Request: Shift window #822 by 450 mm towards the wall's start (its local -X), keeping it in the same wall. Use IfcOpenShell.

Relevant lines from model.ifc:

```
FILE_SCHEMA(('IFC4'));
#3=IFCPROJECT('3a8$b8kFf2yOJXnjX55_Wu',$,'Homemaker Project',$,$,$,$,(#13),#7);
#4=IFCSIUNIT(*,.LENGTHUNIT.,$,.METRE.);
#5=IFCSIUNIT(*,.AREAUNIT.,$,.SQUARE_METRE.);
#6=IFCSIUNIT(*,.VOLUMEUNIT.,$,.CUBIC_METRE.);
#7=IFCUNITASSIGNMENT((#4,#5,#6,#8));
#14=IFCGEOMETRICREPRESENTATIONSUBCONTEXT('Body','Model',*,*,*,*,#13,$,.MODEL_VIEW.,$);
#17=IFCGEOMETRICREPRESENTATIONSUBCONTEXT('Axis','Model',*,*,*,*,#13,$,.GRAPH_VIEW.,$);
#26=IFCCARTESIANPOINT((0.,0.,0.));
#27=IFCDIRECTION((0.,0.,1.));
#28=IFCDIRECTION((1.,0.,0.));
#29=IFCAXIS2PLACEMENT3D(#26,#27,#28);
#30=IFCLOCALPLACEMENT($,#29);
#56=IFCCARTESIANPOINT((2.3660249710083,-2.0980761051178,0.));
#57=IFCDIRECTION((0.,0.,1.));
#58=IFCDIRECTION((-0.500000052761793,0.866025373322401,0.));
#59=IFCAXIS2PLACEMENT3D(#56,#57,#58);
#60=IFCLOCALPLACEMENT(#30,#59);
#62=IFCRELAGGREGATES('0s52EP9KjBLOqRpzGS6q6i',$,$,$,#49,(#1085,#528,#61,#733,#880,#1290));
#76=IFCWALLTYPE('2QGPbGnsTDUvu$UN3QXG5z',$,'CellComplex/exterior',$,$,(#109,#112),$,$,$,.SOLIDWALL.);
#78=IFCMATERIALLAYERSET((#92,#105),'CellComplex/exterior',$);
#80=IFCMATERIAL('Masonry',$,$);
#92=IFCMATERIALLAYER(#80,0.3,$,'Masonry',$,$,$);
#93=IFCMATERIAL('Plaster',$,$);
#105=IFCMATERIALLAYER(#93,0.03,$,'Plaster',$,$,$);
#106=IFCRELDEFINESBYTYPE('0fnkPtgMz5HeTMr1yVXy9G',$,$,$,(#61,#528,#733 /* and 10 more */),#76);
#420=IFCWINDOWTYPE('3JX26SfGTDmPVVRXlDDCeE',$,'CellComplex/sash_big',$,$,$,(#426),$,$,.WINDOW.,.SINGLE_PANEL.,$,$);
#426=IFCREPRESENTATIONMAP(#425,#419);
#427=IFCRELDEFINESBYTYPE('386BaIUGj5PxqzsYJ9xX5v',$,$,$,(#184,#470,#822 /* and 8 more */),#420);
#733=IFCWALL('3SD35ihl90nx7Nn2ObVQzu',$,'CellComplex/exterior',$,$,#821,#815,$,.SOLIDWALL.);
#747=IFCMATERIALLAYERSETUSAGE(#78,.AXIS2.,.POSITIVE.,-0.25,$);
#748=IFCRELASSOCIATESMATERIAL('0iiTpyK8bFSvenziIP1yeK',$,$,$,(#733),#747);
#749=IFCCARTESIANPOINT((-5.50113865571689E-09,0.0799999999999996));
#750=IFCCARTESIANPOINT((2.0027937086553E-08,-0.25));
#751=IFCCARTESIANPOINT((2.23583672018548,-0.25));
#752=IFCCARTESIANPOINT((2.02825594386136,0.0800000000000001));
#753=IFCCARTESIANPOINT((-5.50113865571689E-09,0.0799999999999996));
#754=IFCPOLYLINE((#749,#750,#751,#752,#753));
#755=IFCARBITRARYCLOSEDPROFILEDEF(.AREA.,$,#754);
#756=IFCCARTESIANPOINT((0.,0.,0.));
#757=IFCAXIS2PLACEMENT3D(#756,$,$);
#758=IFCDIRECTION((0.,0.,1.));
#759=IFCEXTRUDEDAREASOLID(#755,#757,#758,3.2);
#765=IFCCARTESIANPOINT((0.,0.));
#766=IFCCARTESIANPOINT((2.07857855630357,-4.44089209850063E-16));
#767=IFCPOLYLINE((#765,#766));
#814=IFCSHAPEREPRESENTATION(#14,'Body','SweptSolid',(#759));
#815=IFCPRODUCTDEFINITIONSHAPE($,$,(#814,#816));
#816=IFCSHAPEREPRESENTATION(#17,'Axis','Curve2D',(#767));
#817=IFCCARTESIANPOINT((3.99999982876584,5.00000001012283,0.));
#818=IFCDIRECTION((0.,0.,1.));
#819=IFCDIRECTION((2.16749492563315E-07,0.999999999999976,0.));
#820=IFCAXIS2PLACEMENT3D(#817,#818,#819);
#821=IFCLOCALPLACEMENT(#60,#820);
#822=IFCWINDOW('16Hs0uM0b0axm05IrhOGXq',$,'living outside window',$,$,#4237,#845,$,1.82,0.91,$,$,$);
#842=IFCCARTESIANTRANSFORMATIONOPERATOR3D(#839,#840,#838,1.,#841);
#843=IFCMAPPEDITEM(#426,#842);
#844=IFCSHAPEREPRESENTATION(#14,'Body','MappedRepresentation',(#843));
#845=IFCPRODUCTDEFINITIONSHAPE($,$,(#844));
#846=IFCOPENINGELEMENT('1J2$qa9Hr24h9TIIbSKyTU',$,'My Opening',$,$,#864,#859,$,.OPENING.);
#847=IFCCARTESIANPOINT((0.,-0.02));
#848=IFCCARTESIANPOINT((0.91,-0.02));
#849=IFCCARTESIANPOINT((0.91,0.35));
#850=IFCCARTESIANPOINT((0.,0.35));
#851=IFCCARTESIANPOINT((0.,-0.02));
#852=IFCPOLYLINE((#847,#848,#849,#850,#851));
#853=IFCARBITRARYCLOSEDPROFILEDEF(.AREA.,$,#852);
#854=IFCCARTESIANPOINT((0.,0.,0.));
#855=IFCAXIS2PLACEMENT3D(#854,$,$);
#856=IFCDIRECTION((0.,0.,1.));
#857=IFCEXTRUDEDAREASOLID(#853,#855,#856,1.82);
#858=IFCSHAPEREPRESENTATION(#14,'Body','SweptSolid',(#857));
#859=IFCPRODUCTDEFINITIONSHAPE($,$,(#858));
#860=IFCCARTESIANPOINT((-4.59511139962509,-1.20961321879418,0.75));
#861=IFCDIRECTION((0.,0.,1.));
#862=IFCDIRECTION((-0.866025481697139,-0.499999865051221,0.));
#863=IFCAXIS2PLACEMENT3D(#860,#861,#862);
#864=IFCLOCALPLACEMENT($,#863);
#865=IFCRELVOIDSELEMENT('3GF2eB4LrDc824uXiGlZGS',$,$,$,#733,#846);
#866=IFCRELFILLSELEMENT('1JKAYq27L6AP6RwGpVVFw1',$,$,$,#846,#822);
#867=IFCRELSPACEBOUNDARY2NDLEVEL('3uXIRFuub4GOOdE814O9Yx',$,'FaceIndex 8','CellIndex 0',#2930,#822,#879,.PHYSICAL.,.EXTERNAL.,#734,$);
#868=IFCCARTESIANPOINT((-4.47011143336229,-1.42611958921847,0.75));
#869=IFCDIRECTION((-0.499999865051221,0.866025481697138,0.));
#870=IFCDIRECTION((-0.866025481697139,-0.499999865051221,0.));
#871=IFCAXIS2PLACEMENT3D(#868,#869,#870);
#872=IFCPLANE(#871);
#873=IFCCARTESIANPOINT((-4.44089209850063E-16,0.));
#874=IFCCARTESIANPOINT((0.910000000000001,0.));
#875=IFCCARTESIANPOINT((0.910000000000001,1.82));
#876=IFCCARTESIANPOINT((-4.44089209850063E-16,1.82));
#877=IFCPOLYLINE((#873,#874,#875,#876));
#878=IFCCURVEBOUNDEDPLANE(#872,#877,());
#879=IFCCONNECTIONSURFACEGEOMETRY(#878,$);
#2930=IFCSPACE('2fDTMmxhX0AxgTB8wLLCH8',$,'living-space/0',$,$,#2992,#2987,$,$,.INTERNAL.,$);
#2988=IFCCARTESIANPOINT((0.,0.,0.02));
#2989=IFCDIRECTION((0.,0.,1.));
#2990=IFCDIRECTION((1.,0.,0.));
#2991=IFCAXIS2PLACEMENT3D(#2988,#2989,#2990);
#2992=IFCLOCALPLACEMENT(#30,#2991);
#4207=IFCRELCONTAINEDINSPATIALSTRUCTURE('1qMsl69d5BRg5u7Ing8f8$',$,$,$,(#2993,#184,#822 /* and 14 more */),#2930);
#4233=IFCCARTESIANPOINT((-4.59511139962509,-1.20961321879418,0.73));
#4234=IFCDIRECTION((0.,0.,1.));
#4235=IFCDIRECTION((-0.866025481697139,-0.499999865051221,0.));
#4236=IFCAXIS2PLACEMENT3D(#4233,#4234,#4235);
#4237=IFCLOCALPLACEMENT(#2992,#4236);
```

```python
import numpy as np
import ifcopenshell
import ifcopenshell.api.geometry
import ifcopenshell.util.placement
import ifcopenshell.util.unit

model = ifcopenshell.open("model.ifc")
unit_scale = ifcopenshell.util.unit.calculate_unit_scale(model)

window = model.by_guid("16Hs0uM0b0axm05IrhOGXq")
opening = window.FillsVoids[0].RelatingOpeningElement
wall = opening.VoidsElements[0].RelatingBuildingElement

wall_matrix = ifcopenshell.util.placement.get_local_placement(wall.ObjectPlacement)
shift = wall_matrix[:3, 0] * -0.45 / unit_scale
before = ifcopenshell.util.placement.get_local_placement(window.ObjectPlacement)[:3, 3].copy()

# The window is not placed relative to its opening, so move both.
for product in (opening, window):
    matrix = ifcopenshell.util.placement.get_local_placement(product.ObjectPlacement)
    matrix[:3, 3] += shift
    ifcopenshell.api.geometry.edit_object_placement(model, product=product, matrix=matrix, is_si=False)

# Space boundary surfaces are stored in each space's coordinates; move them too.
for rel in window.ProvidesBoundaries:
    if not rel.ConnectionGeometry:
        continue
    surface = rel.ConnectionGeometry.SurfaceOnRelatingElement.BasisSurface
    space_matrix = ifcopenshell.util.placement.get_local_placement(rel.RelatingSpace.ObjectPlacement)
    point = np.array(surface.Position.Location.Coordinates) + space_matrix[:3, :3].T @ shift
    surface.Position = model.createIfcAxis2Placement3D(
        model.createIfcCartesianPoint(point.tolist()), surface.Position.Axis, surface.Position.RefDirection
    )

after = ifcopenshell.util.placement.get_local_placement(window.ObjectPlacement)[:3, 3]
print("window moved by", (after - before).round(3) + 0.0)

model.write("model_v2.ifc")
```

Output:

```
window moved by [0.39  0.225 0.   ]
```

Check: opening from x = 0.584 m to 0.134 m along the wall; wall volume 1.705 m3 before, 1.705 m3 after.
